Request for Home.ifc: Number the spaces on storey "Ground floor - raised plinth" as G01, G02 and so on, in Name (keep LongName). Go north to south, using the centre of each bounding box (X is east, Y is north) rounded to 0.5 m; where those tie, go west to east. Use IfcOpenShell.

First a look at what the model holds.

```python
import ifcopenshell
import ifcopenshell.util.element
import ifcopenshell.util.placement

model = ifcopenshell.open("Home.ifc")
print(model.schema)
storey = next(s for s in model.by_type("IfcBuildingStorey") if s.Name == "Ground floor - raised plinth")
spaces = [e for e in ifcopenshell.util.element.get_decomposition(storey) if e.is_a("IfcSpace")]
for e in sorted(spaces, key=lambda e: e.id()):
    origin = ifcopenshell.util.placement.get_local_placement(e.ObjectPlacement)[:3, 3]
    print(e.id(), e.Name, e.LongName, origin.round(2) + 0.0, sep=" | ")
```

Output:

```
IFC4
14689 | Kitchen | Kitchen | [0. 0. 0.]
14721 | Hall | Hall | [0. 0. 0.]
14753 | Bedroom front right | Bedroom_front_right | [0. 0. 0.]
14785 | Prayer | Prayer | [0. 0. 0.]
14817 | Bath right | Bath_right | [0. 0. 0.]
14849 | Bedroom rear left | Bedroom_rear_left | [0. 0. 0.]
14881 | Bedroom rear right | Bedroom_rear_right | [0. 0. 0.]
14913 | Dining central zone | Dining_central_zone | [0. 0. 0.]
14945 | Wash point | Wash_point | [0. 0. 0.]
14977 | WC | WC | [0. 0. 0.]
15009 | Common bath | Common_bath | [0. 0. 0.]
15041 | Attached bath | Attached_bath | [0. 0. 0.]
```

```python
import ifcopenshell
import ifcopenshell.geom
import ifcopenshell.util.element
import ifcopenshell.util.shape

model = ifcopenshell.open("Home.ifc")
settings = ifcopenshell.geom.settings()
settings.set("use-world-coords", True)


def centre(element):
    shape = ifcopenshell.geom.create_shape(settings, element)
    return ifcopenshell.util.shape.get_bbox_centroid(shape.geometry)


storey = next(s for s in model.by_type("IfcBuildingStorey") if s.Name == "Ground floor - raised plinth")
spaces = [e for e in ifcopenshell.util.element.get_decomposition(storey) if e.is_a("IfcSpace")]

# Insertion points can sit at a corner or the storey origin, so sort by the geometry (in metres).
centres = {e: centre(e) for e in spaces}
spaces.sort(key=lambda e: (-round(centres[e][1] / 0.5), centres[e][0]))

for i, e in enumerate(spaces, start=1):
    number = f"G{i:02d}"
    e.Name = number
    print(e.id(), number)

model.write("Home_edited.ifc")
```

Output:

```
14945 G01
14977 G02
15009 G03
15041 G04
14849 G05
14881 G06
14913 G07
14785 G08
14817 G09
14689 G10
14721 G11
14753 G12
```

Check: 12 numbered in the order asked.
